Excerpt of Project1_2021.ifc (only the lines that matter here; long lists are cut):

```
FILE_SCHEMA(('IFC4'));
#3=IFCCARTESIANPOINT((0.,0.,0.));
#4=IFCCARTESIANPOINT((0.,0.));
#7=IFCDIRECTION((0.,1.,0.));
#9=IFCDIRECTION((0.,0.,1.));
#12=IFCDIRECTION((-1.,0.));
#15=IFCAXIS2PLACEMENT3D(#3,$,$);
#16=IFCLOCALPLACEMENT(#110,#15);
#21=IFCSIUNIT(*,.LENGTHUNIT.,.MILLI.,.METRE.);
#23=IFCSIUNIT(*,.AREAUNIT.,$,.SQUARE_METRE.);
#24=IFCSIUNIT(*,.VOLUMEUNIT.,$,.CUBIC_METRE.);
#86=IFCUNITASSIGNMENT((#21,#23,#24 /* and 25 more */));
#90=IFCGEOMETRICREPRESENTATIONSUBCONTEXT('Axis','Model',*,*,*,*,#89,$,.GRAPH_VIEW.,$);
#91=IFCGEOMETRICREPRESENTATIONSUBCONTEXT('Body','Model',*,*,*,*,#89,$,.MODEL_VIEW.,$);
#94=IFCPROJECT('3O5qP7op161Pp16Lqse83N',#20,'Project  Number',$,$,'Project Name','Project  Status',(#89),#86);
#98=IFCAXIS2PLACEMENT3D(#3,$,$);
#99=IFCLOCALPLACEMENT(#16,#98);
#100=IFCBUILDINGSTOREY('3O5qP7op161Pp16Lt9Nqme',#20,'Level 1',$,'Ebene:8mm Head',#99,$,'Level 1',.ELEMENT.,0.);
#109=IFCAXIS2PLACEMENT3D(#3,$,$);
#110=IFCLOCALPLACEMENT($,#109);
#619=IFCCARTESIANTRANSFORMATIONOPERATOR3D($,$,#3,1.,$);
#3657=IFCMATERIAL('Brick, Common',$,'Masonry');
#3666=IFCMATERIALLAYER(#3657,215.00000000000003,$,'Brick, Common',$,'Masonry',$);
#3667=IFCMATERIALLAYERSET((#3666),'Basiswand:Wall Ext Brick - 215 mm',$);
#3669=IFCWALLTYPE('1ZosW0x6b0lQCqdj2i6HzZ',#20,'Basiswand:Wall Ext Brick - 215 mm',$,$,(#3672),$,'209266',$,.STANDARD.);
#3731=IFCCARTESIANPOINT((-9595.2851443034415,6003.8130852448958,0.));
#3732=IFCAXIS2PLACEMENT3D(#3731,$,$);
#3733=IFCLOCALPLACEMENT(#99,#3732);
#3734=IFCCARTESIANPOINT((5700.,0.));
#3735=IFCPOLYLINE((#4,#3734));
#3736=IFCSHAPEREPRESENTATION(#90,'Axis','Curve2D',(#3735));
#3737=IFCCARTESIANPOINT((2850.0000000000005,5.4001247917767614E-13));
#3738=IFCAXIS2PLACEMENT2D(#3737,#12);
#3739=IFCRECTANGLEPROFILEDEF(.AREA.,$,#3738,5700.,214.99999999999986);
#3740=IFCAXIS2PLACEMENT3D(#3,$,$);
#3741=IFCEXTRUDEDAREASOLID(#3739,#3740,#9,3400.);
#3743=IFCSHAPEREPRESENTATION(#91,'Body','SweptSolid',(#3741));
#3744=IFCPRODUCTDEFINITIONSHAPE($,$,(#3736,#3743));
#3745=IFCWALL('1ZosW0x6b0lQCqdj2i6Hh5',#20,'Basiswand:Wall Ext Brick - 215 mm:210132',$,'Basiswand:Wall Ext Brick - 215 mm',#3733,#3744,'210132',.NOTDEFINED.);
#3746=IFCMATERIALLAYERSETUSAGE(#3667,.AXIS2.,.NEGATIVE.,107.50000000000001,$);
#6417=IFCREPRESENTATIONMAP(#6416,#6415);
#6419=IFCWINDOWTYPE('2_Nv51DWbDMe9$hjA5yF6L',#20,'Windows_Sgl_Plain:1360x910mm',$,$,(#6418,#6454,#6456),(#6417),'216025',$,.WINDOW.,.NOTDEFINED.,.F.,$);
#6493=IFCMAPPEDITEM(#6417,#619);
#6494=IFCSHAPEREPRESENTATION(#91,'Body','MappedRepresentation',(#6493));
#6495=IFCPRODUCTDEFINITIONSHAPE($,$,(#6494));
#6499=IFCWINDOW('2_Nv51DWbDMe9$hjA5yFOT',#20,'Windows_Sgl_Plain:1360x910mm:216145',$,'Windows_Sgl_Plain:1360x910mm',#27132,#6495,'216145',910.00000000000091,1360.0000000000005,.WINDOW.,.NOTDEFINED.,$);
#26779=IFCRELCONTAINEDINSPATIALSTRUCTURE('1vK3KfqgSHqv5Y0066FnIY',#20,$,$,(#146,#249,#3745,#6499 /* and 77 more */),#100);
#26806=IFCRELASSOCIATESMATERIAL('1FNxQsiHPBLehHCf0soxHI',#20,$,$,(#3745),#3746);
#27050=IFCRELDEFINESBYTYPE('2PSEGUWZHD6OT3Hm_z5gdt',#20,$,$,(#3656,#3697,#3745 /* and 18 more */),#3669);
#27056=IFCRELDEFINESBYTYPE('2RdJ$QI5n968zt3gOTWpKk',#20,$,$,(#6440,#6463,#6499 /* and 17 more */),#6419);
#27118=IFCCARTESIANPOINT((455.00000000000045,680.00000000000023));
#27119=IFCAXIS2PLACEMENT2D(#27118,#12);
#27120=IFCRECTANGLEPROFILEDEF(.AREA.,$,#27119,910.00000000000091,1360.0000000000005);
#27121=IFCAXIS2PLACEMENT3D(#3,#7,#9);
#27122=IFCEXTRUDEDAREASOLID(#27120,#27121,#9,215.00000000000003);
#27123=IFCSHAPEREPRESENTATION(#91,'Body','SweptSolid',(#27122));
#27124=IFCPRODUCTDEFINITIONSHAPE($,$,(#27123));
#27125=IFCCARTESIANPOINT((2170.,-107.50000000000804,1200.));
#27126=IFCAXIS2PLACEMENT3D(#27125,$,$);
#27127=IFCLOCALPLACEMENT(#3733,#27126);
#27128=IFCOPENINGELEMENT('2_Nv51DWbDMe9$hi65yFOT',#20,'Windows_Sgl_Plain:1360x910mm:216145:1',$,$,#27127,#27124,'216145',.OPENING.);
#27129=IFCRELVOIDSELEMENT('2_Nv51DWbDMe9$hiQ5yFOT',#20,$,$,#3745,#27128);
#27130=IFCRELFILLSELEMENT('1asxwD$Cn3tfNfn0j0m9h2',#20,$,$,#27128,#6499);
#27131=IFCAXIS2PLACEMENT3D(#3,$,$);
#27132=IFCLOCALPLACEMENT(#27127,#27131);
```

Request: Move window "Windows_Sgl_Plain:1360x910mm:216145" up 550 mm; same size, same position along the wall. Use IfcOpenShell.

```python
import numpy as np
import ifcopenshell
import ifcopenshell.api.geometry
import ifcopenshell.util.placement
import ifcopenshell.util.unit

model = ifcopenshell.open("Project1_2021.ifc")
unit_scale = ifcopenshell.util.unit.calculate_unit_scale(model)

window = model.by_guid("2_Nv51DWbDMe9$hjA5yFOT")
opening = window.FillsVoids[0].RelatingOpeningElement
dz = 0.55 / unit_scale

shift = np.array([0.0, 0.0, dz])
# The window is placed relative to its opening, so it follows when the opening moves.
matrix = ifcopenshell.util.placement.get_local_placement(opening.ObjectPlacement)
matrix[:3, 3] += shift
ifcopenshell.api.geometry.edit_object_placement(
    model, product=opening, matrix=matrix, is_si=False, should_transform_children=True
)

print(f"moved by {dz * unit_scale:+.3f} m")

model.write("Project1_2021_edited.ifc")
```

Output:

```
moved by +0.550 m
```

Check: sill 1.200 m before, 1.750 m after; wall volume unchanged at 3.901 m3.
